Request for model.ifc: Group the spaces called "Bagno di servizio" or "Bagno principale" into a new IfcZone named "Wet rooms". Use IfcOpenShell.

First a look at what the model holds.

```python
import ifcopenshell

model = ifcopenshell.open("model.ifc")
print(model.schema)
seen = {}
for space in model.by_type("IfcSpace"):
    seen[space.LongName] = seen.get(space.LongName, 0) + 1
for name, count in sorted(seen.items(), key=str):
    print(count, "x", name)
print("zones:", [z.Name for z in model.by_type("IfcZone")][:20])
```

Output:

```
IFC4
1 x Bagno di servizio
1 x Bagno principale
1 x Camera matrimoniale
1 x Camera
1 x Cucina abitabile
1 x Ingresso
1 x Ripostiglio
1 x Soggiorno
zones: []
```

```python
import ifcopenshell
import ifcopenshell.api.group
import ifcopenshell.api.root

model = ifcopenshell.open("model.ifc")

names = {"Bagno di servizio", "Bagno principale"}
spaces = [s for s in model.by_type("IfcSpace") if s.LongName in names]

zone = ifcopenshell.api.root.create_entity(model, ifc_class="IfcZone", name="Wet rooms")
ifcopenshell.api.group.assign_group(model, products=spaces, group=zone)
print(len(spaces), "spaces in", zone.Name)

model.write("model_rev.ifc")
```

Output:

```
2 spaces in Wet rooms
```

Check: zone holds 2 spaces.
